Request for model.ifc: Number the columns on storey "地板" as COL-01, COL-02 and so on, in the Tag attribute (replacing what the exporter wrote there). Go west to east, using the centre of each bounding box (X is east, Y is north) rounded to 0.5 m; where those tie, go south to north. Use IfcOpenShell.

First a look at what the model holds.

```python
import ifcopenshell
import ifcopenshell.util.element
import ifcopenshell.util.placement

model = ifcopenshell.open("model.ifc")
print(model.schema)
storey = next(s for s in model.by_type("IfcBuildingStorey") if s.Name == "地板")
columns = [e for e in ifcopenshell.util.element.get_decomposition(storey) if e.is_a("IfcColumn")]
for e in sorted(columns, key=lambda e: e.id()):
    origin = ifcopenshell.util.placement.get_local_placement(e.ObjectPlacement)[:3, 3]
    print(e.id(), e.Tag, e.Name, origin.round(2) + 0.0, sep=" | ")
```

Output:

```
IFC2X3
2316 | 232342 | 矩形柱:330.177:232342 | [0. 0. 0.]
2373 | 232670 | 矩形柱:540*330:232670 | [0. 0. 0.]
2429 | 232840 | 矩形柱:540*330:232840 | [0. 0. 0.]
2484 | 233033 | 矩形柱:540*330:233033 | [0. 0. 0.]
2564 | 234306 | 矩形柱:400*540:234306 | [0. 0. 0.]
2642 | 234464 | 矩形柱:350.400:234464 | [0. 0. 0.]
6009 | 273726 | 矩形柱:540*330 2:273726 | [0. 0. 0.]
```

```python
import ifcopenshell
import ifcopenshell.geom
import ifcopenshell.util.element
import ifcopenshell.util.shape

model = ifcopenshell.open("model.ifc")
settings = ifcopenshell.geom.settings()
settings.set("use-world-coords", True)


def centre(element):
    shape = ifcopenshell.geom.create_shape(settings, element)
    return ifcopenshell.util.shape.get_bbox_centroid(shape.geometry)


storey = next(s for s in model.by_type("IfcBuildingStorey") if s.Name == "地板")
columns = [e for e in ifcopenshell.util.element.get_decomposition(storey) if e.is_a("IfcColumn")]

# Insertion points can sit at a corner or the storey origin, so sort by the geometry (in metres).
centres = {e: centre(e) for e in columns}
columns.sort(key=lambda e: (round(centres[e][0] / 0.5), centres[e][1]))

for i, e in enumerate(columns, start=1):
    number = f"COL-{i:02d}"
    e.Tag = number
    print(e.id(), number)

model.write("model_v2.ifc")
```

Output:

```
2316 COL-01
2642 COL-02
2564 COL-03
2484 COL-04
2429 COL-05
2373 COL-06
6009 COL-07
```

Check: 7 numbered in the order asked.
